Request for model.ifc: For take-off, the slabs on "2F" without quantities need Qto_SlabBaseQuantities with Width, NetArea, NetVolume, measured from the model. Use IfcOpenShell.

First a look at what the model holds.

```python
import ifcopenshell
import ifcopenshell.util.element
import ifcopenshell.util.unit

model = ifcopenshell.open("model.ifc")
print(model.schema)
for unit_type in ("LENGTHUNIT", "AREAUNIT", "VOLUMEUNIT"):
    print(unit_type, ifcopenshell.util.unit.calculate_unit_scale(model, unit_type))
storey = next(s for s in model.by_type("IfcBuildingStorey") if s.Name == "2F")
slabs = [e for e in ifcopenshell.util.element.get_decomposition(storey) if e.is_a("IfcSlab")]
for e in sorted(slabs, key=lambda e: e.id()):
    print(e.id(), e.is_a(), e.Name, list(ifcopenshell.util.element.get_psets(e, qtos_only=True)), sep=" | ")
```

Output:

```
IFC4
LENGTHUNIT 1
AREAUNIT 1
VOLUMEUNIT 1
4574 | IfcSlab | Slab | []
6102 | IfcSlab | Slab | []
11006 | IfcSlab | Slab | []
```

```python
import ifcopenshell
import ifcopenshell.api.pset
import ifcopenshell.geom
import ifcopenshell.util.element
import ifcopenshell.util.shape
import ifcopenshell.util.unit

model = ifcopenshell.open("model.ifc")
unit_scale = ifcopenshell.util.unit.calculate_unit_scale(model)
area_scale = ifcopenshell.util.unit.calculate_unit_scale(model, "AREAUNIT")
volume_scale = ifcopenshell.util.unit.calculate_unit_scale(model, "VOLUMEUNIT")
settings = ifcopenshell.geom.settings()

storey = next(s for s in model.by_type("IfcBuildingStorey") if s.Name == "2F")
slabs = [e for e in ifcopenshell.util.element.get_decomposition(storey) if e.is_a("IfcSlab")]

for e in sorted(slabs, key=lambda e: e.id()):
    if ifcopenshell.util.element.get_psets(e, qtos_only=True, should_inherit=False):
        continue
    # Geometry comes back in metres, in the element's own axes.
    shape = ifcopenshell.geom.create_shape(settings, e)
    values = {
        "Width": ifcopenshell.util.shape.get_z(shape.geometry) / unit_scale,
        "NetArea": ifcopenshell.util.shape.get_footprint_area(shape.geometry) / area_scale,
        "NetVolume": ifcopenshell.util.shape.get_volume(shape.geometry) / volume_scale,
    }
    qto = ifcopenshell.api.pset.add_qto(model, product=e, name="Qto_SlabBaseQuantities")
    ifcopenshell.api.pset.edit_qto(model, qto=qto, properties=values)
    print(e.id(), {k: round(v, 3) for k, v in values.items()})

model.write("model_edited.ifc")
```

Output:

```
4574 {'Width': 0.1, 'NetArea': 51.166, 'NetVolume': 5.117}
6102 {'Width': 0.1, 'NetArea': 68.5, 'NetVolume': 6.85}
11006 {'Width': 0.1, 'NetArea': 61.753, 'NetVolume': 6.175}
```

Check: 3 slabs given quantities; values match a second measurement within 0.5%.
